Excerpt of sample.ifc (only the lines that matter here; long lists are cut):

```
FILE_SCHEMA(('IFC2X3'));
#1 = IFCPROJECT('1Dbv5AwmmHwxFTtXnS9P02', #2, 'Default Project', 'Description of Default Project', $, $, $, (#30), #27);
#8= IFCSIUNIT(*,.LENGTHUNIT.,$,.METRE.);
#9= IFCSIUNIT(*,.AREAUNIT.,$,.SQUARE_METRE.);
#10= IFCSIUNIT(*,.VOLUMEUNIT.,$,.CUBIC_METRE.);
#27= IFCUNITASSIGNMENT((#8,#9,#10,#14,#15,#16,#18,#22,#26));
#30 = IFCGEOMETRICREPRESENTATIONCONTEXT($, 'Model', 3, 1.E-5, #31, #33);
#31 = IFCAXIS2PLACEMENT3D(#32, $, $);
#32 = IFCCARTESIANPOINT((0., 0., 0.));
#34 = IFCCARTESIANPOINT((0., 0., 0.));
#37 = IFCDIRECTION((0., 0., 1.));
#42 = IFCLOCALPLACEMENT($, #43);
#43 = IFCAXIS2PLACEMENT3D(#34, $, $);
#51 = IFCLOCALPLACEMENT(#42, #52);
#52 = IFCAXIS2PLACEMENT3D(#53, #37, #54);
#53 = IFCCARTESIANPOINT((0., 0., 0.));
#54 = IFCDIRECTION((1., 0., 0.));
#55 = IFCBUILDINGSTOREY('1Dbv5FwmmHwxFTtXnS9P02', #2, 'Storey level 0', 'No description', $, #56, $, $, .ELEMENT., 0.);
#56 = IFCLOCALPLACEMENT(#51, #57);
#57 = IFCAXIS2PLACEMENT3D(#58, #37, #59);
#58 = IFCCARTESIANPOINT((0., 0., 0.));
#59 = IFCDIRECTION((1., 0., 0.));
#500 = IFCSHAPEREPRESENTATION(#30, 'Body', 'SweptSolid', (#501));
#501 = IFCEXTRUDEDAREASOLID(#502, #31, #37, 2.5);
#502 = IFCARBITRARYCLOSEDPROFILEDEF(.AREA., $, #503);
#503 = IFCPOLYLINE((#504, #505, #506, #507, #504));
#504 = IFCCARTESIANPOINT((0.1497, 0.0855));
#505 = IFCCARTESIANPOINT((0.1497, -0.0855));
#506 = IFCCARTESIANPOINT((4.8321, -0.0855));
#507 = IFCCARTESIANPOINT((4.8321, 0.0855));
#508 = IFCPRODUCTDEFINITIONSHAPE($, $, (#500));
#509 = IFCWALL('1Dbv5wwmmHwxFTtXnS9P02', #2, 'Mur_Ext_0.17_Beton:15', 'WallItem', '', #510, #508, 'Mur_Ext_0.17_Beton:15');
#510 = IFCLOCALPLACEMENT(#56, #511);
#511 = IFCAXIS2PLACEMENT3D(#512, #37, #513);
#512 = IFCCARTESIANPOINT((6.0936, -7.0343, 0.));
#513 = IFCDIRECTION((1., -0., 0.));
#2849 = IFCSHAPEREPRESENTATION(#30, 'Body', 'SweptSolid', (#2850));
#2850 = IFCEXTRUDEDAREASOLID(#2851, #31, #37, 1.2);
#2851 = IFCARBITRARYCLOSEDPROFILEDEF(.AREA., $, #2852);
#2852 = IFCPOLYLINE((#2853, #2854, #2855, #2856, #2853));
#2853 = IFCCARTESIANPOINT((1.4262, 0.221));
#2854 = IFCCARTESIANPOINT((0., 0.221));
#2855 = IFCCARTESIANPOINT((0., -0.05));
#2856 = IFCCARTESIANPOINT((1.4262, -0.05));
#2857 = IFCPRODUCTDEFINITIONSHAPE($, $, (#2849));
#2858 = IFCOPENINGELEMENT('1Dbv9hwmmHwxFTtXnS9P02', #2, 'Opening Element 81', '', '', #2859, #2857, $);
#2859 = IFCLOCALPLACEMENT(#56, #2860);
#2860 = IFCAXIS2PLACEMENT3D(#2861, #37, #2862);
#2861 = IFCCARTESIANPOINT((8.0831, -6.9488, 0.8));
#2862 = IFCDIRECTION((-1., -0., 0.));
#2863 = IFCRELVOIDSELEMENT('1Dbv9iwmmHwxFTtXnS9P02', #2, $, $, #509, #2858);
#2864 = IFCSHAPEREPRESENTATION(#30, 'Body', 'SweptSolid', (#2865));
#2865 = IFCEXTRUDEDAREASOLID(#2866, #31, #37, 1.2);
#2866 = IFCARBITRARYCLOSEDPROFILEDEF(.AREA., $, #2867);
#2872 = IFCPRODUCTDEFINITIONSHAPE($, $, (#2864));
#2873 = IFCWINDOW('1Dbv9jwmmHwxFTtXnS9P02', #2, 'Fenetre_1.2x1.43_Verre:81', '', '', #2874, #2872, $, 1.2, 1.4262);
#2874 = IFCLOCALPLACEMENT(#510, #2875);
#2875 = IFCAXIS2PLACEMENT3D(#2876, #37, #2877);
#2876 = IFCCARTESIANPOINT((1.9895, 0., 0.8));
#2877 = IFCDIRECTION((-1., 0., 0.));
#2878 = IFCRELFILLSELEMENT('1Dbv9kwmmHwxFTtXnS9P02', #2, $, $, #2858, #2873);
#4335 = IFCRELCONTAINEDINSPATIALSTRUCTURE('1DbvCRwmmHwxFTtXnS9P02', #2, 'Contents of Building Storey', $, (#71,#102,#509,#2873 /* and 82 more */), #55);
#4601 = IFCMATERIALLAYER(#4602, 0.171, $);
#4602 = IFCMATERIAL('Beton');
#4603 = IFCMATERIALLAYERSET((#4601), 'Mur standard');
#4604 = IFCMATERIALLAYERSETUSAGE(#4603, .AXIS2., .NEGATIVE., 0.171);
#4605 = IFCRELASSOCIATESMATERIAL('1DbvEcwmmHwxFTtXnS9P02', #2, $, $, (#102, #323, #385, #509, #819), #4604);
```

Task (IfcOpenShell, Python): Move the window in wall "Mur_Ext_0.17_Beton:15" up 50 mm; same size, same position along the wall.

```python
import numpy as np
import ifcopenshell
import ifcopenshell.api.geometry
import ifcopenshell.util.placement
import ifcopenshell.util.unit

model = ifcopenshell.open("sample.ifc")
unit_scale = ifcopenshell.util.unit.calculate_unit_scale(model)

window = model.by_id(2873)
opening = window.FillsVoids[0].RelatingOpeningElement
dz = 0.05

shift = np.array([0.0, 0.0, dz])
# The window is not placed relative to its opening, so move both.
for product in (opening, window):
    matrix = ifcopenshell.util.placement.get_local_placement(product.ObjectPlacement)
    matrix[:3, 3] += shift
    ifcopenshell.api.geometry.edit_object_placement(model, product=product, matrix=matrix, is_si=False)

print(f"moved by {dz * unit_scale:+.3f} m")

model.write("sample_edited.ifc")
```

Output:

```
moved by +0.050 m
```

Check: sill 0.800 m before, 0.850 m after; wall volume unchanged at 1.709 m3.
